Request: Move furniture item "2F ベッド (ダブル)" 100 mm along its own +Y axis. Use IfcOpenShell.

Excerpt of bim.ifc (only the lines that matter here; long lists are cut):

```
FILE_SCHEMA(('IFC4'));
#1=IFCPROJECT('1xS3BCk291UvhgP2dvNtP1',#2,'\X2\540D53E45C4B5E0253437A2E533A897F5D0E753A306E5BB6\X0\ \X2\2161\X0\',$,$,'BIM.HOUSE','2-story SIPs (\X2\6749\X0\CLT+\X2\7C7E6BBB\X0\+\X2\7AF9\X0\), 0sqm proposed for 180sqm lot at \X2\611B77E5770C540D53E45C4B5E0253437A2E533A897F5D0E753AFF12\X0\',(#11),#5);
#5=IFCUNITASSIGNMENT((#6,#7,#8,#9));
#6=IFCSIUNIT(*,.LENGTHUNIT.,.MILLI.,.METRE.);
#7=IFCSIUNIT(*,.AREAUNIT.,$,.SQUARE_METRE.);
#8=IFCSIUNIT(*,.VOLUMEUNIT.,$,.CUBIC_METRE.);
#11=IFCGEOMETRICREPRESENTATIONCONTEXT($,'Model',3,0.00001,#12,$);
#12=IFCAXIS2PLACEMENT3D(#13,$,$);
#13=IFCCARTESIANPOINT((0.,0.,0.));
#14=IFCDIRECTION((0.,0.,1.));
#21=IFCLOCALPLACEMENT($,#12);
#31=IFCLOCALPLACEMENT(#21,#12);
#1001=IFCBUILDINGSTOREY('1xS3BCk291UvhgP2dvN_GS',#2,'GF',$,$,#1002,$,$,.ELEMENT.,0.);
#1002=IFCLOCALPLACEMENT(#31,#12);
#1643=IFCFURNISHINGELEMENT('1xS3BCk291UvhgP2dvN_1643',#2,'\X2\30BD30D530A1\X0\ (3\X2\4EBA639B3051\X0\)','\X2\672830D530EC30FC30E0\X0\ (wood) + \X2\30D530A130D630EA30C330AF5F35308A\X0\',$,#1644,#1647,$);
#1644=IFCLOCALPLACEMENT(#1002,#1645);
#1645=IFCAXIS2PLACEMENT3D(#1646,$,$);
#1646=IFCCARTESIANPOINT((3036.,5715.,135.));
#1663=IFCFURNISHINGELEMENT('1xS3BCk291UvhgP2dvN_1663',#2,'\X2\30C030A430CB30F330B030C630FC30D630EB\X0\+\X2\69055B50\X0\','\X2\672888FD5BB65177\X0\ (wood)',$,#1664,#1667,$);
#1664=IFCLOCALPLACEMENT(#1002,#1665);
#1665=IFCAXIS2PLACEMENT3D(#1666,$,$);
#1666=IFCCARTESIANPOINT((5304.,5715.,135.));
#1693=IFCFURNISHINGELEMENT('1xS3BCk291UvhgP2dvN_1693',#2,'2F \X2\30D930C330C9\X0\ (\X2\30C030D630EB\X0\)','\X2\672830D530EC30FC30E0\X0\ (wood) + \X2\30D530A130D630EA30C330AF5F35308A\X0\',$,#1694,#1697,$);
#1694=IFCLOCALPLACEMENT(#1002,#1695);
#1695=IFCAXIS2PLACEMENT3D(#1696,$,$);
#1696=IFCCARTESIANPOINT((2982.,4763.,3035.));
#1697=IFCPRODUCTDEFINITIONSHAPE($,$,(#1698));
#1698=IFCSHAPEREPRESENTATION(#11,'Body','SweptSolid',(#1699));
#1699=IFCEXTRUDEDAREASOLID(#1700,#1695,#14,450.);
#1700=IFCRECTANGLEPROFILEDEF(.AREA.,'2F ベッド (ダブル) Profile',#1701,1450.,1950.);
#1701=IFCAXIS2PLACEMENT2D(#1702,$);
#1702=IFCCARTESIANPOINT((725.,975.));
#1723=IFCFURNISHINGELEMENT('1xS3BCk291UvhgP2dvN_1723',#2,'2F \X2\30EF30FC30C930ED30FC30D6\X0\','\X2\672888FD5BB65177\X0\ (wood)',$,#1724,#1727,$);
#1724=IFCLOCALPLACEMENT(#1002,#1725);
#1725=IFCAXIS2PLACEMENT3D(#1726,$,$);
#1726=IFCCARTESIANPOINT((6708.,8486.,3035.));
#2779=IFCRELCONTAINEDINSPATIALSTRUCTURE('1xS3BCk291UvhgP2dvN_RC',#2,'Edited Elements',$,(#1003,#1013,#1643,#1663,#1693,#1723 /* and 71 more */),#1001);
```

```python
import ifcopenshell
import ifcopenshell.api.geometry
import ifcopenshell.util.placement
import ifcopenshell.util.unit

model = ifcopenshell.open("bim.ifc")
unit_scale = ifcopenshell.util.unit.calculate_unit_scale(model)

item = model.by_guid("1xS3BCk291UvhgP2dvN_1693")
matrix = ifcopenshell.util.placement.get_local_placement(item.ObjectPlacement)
matrix[:3, 3] += matrix[:3, 1] * 0.1 / unit_scale
ifcopenshell.api.geometry.edit_object_placement(model, product=item, matrix=matrix, is_si=False)

print(ifcopenshell.util.placement.get_local_placement(item.ObjectPlacement).round(3) + 0.0)

model.write("bim_edited.ifc")
```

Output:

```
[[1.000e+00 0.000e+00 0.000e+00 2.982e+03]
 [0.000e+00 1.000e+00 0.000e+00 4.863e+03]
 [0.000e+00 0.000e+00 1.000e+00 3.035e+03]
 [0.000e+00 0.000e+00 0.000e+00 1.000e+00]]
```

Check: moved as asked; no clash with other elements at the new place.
